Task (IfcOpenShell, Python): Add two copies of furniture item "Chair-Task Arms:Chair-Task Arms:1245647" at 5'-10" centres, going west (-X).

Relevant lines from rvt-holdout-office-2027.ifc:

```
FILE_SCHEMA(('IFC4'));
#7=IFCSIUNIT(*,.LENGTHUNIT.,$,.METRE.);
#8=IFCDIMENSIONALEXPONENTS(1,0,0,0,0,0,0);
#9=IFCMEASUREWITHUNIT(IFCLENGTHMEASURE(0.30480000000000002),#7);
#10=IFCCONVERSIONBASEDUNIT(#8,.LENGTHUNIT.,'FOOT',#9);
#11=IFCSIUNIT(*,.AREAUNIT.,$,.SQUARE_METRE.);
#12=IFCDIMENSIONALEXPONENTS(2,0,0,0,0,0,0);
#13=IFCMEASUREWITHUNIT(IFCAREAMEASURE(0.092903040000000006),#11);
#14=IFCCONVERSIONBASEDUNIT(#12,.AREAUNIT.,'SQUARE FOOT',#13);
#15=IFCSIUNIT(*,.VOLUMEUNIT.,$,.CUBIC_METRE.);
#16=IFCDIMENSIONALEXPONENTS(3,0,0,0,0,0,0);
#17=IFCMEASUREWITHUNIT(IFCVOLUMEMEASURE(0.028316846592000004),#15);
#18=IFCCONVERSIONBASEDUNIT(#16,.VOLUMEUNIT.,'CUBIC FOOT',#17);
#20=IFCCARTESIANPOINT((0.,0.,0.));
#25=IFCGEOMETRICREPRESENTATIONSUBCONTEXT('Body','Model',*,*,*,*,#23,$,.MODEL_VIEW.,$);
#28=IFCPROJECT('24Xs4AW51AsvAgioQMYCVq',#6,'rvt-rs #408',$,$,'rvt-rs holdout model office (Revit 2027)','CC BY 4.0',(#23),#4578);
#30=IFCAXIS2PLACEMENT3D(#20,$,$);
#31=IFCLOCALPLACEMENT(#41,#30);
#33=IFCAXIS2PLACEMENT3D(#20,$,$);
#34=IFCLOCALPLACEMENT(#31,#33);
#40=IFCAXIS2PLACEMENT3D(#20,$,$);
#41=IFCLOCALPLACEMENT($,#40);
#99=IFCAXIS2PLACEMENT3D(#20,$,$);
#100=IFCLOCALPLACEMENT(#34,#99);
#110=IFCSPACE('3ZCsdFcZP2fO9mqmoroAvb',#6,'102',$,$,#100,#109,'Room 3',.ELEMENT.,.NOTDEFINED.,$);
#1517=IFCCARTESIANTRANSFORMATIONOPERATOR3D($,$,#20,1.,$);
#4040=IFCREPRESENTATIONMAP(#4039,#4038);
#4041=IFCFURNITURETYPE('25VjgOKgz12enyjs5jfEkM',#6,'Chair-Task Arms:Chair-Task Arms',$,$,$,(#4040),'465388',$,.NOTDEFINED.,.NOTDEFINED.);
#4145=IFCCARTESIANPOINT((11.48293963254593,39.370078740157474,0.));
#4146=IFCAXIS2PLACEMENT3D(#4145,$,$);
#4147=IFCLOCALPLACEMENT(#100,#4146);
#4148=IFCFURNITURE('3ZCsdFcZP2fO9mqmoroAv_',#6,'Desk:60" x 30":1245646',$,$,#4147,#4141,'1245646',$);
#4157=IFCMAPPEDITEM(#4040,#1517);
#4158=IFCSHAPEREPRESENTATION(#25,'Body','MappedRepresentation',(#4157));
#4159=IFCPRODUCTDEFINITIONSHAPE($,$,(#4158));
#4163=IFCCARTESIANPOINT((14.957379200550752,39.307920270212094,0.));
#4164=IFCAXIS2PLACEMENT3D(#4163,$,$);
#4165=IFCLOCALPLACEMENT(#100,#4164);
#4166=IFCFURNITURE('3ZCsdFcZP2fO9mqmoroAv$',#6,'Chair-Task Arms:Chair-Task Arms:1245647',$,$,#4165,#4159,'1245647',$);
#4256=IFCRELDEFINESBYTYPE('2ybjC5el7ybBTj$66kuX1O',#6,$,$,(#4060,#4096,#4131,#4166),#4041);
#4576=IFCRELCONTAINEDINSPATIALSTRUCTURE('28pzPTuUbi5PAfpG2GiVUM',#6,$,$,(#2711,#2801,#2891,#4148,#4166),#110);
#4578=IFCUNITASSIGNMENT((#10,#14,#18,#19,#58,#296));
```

```python
import numpy as np
import ifcopenshell
import ifcopenshell.api.geometry
import ifcopenshell.api.root
import ifcopenshell.util.element
import ifcopenshell.util.placement
import ifcopenshell.util.unit

model = ifcopenshell.open("rvt-holdout-office-2027.ifc")
unit_scale = ifcopenshell.util.unit.calculate_unit_scale(model)


def reuse_history(source, copy):
    """copy_class also copies each property set's owner history, people and application; keep the originals."""
    for rel in copy.IsDefinedBy:
        if rel.is_a("IfcRelDefinesByProperties") and (history := rel.RelatingPropertyDefinition.OwnerHistory):
            rel.RelatingPropertyDefinition.OwnerHistory = source.OwnerHistory
            ifcopenshell.util.element.remove_deep2(model, history)


source = model.by_id(4166)
base = ifcopenshell.util.placement.get_local_placement(source.ObjectPlacement)
step = np.array([-1.0, 0.0, 0.0]) * 70 * 0.0254 / unit_scale

for i in range(1, 3):
    copy = ifcopenshell.api.root.copy_class(model, product=source)
    copy.Representation = ifcopenshell.util.element.copy_deep(
        model, source.Representation, exclude=["IfcGeometricRepresentationContext", "IfcRepresentationMap"]
    )
    copy.Name = "Chair-Task Arms:Chair-Task Arms"
    copy.Tag = None
    reuse_history(source, copy)
    matrix = base.copy()
    matrix[:3, 3] += i * step
    print("added at", matrix[:3, 3].round(3) + 0.0)
    ifcopenshell.api.geometry.edit_object_placement(model, product=copy, matrix=matrix, is_si=False)

model.write("rvt-holdout-office-2027_updated.ifc")
```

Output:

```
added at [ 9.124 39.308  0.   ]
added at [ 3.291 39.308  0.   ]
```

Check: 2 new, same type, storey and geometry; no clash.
